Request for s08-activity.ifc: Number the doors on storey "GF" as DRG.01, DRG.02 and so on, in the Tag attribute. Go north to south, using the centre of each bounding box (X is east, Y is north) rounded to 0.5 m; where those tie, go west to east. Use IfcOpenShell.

First a look at what the model holds.

```python
import ifcopenshell
import ifcopenshell.util.element
import ifcopenshell.util.placement

model = ifcopenshell.open("s08-activity.ifc")
print(model.schema)
storey = next(s for s in model.by_type("IfcBuildingStorey") if s.Name == "GF")
doors = [e for e in ifcopenshell.util.element.get_decomposition(storey) if e.is_a("IfcDoor")]
for e in sorted(doors, key=lambda e: e.id()):
    origin = ifcopenshell.util.placement.get_local_placement(e.ObjectPlacement)[:3, 3]
    print(e.id(), e.Tag, e.Name, origin.round(2) + 0.0, sep=" | ")
```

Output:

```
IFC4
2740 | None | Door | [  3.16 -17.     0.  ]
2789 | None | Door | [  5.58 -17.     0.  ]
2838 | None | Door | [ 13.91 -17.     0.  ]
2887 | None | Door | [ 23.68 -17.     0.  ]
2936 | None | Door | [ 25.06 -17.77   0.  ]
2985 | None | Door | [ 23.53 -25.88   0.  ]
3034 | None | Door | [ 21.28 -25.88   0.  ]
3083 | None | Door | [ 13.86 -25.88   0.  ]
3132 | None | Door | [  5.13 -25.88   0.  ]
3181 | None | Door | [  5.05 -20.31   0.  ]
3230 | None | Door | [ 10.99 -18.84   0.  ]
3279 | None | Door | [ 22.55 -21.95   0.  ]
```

```python
import ifcopenshell
import ifcopenshell.geom
import ifcopenshell.util.element
import ifcopenshell.util.shape

model = ifcopenshell.open("s08-activity.ifc")
settings = ifcopenshell.geom.settings()
settings.set("use-world-coords", True)


def centre(element):
    shape = ifcopenshell.geom.create_shape(settings, element)
    return ifcopenshell.util.shape.get_bbox_centroid(shape.geometry)


storey = next(s for s in model.by_type("IfcBuildingStorey") if s.Name == "GF")
doors = [e for e in ifcopenshell.util.element.get_decomposition(storey) if e.is_a("IfcDoor")]

# Insertion points can sit at a corner or the storey origin, so sort by the geometry (in metres).
centres = {e: centre(e) for e in doors}
doors.sort(key=lambda e: (-round(centres[e][1] / 0.5), centres[e][0]))

for i, e in enumerate(doors, start=1):
    number = f"DRG.{i:02d}"
    e.Tag = number
    print(e.id(), number)

model.write("s08-activity-out.ifc")
```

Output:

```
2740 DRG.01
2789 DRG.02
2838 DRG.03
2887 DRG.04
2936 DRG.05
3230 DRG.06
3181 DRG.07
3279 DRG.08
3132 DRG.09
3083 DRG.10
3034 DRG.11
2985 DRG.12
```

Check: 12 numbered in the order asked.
